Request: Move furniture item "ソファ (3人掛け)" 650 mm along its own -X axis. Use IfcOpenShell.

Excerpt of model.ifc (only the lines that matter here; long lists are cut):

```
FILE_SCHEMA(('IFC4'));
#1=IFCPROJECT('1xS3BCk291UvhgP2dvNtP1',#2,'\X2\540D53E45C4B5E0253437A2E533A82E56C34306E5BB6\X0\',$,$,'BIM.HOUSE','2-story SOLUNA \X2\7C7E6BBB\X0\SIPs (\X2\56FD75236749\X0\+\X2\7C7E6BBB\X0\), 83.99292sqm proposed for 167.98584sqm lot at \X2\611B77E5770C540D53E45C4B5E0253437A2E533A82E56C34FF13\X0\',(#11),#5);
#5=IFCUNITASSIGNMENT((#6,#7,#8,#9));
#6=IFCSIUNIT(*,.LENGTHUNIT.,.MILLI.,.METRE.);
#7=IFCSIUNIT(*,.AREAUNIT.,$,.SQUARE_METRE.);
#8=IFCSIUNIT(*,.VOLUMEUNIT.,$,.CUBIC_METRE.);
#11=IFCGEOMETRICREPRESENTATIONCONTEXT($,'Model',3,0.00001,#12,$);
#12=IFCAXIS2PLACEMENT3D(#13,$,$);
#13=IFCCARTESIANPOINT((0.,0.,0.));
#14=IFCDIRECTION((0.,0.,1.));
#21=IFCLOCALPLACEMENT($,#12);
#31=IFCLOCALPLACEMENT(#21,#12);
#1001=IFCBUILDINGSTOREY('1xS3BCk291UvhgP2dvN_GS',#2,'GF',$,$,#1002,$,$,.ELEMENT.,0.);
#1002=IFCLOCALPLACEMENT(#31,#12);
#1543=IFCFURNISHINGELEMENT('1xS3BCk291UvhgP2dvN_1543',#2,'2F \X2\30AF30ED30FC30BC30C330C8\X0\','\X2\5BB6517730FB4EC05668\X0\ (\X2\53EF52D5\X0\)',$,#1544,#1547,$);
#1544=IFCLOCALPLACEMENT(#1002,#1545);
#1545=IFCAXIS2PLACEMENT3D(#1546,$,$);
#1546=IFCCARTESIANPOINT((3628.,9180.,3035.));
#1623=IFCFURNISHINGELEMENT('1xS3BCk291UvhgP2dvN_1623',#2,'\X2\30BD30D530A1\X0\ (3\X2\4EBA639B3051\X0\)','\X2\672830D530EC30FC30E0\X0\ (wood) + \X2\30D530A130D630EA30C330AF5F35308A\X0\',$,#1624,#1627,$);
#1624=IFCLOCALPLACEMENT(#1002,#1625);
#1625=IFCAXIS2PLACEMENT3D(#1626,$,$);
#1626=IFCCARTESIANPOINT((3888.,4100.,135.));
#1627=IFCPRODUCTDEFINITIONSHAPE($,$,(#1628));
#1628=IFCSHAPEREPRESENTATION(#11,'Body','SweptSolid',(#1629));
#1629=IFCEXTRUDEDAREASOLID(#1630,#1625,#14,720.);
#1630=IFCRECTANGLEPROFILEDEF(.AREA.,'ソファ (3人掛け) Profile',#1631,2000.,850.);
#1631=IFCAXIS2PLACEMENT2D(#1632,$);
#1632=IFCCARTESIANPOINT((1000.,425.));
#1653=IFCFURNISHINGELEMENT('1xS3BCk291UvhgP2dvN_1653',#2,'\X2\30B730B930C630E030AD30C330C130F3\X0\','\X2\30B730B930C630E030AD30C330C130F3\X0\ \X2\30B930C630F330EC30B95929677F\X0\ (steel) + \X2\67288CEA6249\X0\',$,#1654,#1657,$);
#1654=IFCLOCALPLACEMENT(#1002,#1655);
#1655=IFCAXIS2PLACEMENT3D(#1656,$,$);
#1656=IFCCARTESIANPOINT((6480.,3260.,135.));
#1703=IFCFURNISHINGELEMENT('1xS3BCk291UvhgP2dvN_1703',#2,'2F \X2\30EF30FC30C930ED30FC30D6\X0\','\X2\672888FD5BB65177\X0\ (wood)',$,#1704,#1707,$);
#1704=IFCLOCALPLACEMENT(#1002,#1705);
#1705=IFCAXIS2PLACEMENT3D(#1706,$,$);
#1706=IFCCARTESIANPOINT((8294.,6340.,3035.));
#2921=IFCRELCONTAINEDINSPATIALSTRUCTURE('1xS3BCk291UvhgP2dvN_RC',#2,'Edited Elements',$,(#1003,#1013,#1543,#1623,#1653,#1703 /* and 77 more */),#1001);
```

```python
import ifcopenshell
import ifcopenshell.api.geometry
import ifcopenshell.util.placement

model = ifcopenshell.open("model.ifc")

item = model.by_guid("1xS3BCk291UvhgP2dvN_1623")
matrix = ifcopenshell.util.placement.get_local_placement(item.ObjectPlacement)
matrix[:3, 3] -= matrix[:3, 0] * 650.0
ifcopenshell.api.geometry.edit_object_placement(model, product=item, matrix=matrix, is_si=False)

print(ifcopenshell.util.placement.get_local_placement(item.ObjectPlacement).round(3) + 0.0)

model.write("model_edited.ifc")
```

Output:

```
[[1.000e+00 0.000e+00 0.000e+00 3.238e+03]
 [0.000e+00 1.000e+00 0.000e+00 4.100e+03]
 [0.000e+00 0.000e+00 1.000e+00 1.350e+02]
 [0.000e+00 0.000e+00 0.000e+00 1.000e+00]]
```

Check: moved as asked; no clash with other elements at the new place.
